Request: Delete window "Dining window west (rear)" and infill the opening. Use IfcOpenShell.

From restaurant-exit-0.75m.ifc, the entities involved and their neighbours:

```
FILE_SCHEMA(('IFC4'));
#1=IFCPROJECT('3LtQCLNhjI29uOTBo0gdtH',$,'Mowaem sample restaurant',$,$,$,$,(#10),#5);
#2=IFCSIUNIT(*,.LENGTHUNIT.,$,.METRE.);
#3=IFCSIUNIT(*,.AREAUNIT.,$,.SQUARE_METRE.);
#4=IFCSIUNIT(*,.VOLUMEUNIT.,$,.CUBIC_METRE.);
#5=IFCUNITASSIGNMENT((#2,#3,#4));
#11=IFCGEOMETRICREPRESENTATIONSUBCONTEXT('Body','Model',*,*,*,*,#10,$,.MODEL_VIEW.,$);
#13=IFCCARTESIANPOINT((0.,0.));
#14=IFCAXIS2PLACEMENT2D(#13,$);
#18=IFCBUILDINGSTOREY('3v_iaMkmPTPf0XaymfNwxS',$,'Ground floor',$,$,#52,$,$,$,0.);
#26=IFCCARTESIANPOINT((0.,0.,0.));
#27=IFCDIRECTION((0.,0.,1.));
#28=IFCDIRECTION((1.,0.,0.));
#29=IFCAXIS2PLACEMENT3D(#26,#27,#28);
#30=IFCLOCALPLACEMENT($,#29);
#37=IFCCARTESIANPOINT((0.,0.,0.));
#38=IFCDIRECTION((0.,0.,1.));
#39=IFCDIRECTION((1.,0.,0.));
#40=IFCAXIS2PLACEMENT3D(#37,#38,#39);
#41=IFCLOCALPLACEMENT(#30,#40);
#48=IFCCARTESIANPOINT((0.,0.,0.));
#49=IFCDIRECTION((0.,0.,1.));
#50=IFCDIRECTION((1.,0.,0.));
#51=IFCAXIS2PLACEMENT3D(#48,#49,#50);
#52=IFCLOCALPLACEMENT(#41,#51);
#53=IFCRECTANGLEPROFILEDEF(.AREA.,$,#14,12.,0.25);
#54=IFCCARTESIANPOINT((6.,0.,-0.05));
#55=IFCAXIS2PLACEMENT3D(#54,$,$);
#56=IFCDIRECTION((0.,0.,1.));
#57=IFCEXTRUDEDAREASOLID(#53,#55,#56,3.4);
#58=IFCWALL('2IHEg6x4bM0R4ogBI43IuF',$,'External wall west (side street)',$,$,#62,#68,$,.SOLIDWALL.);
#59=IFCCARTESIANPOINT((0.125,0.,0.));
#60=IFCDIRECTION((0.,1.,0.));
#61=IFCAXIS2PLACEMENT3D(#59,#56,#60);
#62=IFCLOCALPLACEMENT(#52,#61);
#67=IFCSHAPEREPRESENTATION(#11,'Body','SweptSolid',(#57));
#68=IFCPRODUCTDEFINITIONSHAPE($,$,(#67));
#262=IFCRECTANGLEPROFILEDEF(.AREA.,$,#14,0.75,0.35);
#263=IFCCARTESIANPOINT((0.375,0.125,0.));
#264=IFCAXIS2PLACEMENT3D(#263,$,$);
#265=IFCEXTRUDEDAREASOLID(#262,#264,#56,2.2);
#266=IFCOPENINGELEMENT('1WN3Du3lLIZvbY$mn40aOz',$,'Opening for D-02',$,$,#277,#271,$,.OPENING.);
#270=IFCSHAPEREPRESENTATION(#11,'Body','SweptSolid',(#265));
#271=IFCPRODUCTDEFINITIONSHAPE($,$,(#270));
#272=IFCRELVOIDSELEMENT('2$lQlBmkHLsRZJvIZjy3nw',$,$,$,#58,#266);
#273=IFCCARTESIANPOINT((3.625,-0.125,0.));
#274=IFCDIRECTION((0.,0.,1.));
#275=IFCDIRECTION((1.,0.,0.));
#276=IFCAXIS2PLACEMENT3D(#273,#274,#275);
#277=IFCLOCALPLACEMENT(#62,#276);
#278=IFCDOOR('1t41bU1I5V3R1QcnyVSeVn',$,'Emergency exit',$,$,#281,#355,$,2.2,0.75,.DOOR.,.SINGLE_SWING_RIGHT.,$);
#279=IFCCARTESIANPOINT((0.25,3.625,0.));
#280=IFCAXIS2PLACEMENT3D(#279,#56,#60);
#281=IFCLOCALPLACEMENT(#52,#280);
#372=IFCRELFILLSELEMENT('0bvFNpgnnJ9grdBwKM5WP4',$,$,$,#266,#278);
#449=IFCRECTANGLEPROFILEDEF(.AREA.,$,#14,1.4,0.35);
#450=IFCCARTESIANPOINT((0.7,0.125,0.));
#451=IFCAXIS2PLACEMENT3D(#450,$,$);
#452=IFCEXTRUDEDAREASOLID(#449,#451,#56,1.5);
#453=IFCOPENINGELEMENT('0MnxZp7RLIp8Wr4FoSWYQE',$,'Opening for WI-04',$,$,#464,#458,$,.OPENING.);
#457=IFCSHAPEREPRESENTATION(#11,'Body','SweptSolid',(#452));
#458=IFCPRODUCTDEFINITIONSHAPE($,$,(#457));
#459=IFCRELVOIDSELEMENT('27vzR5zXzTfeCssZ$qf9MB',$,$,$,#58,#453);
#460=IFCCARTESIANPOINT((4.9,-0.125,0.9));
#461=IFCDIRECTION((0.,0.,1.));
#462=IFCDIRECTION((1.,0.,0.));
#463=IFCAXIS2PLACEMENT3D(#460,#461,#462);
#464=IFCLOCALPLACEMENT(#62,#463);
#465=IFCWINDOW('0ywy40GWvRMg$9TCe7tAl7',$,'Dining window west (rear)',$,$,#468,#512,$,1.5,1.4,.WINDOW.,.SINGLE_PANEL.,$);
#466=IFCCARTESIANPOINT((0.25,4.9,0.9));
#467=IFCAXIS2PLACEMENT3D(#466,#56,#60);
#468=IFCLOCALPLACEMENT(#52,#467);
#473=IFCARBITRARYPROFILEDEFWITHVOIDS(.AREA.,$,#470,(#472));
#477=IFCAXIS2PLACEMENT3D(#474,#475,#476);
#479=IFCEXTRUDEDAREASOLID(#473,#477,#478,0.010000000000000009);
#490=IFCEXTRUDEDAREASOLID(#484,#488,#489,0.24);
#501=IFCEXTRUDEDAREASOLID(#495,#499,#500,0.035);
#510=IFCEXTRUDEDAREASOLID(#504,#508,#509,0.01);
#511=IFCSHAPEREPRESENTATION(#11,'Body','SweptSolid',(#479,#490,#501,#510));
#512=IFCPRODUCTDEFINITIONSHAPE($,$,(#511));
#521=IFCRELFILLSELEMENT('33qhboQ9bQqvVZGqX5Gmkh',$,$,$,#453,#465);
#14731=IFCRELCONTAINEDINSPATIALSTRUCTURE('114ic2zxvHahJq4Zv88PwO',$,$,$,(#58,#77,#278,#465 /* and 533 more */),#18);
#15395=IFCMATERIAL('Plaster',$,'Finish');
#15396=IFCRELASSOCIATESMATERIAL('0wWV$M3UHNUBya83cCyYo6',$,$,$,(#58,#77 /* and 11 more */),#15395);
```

```python
import ifcopenshell
import ifcopenshell.api.feature
import ifcopenshell.api.root
import ifcopenshell.geom
import ifcopenshell.util.shape

model = ifcopenshell.open("restaurant-exit-0.75m.ifc")
settings = ifcopenshell.geom.settings()


def volume(element):
    """Net volume in cubic metres, openings subtracted."""
    shape = ifcopenshell.geom.create_shape(settings, element)
    return ifcopenshell.util.shape.get_volume(shape.geometry)


window = model.by_guid("0ywy40GWvRMg$9TCe7tAl7")
opening = window.FillsVoids[0].RelatingOpeningElement
wall = opening.VoidsElements[0].RelatingBuildingElement
before = volume(wall)

ifcopenshell.api.root.remove_product(model, product=window)
ifcopenshell.api.feature.remove_feature(model, feature=opening)

after = volume(wall)

print(f"wall volume {before:.3f} -> {after:.3f} m3")

model.write("restaurant-exit-0.75m_updated.ifc")
```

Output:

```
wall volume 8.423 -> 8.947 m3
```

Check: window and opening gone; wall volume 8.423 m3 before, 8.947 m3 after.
